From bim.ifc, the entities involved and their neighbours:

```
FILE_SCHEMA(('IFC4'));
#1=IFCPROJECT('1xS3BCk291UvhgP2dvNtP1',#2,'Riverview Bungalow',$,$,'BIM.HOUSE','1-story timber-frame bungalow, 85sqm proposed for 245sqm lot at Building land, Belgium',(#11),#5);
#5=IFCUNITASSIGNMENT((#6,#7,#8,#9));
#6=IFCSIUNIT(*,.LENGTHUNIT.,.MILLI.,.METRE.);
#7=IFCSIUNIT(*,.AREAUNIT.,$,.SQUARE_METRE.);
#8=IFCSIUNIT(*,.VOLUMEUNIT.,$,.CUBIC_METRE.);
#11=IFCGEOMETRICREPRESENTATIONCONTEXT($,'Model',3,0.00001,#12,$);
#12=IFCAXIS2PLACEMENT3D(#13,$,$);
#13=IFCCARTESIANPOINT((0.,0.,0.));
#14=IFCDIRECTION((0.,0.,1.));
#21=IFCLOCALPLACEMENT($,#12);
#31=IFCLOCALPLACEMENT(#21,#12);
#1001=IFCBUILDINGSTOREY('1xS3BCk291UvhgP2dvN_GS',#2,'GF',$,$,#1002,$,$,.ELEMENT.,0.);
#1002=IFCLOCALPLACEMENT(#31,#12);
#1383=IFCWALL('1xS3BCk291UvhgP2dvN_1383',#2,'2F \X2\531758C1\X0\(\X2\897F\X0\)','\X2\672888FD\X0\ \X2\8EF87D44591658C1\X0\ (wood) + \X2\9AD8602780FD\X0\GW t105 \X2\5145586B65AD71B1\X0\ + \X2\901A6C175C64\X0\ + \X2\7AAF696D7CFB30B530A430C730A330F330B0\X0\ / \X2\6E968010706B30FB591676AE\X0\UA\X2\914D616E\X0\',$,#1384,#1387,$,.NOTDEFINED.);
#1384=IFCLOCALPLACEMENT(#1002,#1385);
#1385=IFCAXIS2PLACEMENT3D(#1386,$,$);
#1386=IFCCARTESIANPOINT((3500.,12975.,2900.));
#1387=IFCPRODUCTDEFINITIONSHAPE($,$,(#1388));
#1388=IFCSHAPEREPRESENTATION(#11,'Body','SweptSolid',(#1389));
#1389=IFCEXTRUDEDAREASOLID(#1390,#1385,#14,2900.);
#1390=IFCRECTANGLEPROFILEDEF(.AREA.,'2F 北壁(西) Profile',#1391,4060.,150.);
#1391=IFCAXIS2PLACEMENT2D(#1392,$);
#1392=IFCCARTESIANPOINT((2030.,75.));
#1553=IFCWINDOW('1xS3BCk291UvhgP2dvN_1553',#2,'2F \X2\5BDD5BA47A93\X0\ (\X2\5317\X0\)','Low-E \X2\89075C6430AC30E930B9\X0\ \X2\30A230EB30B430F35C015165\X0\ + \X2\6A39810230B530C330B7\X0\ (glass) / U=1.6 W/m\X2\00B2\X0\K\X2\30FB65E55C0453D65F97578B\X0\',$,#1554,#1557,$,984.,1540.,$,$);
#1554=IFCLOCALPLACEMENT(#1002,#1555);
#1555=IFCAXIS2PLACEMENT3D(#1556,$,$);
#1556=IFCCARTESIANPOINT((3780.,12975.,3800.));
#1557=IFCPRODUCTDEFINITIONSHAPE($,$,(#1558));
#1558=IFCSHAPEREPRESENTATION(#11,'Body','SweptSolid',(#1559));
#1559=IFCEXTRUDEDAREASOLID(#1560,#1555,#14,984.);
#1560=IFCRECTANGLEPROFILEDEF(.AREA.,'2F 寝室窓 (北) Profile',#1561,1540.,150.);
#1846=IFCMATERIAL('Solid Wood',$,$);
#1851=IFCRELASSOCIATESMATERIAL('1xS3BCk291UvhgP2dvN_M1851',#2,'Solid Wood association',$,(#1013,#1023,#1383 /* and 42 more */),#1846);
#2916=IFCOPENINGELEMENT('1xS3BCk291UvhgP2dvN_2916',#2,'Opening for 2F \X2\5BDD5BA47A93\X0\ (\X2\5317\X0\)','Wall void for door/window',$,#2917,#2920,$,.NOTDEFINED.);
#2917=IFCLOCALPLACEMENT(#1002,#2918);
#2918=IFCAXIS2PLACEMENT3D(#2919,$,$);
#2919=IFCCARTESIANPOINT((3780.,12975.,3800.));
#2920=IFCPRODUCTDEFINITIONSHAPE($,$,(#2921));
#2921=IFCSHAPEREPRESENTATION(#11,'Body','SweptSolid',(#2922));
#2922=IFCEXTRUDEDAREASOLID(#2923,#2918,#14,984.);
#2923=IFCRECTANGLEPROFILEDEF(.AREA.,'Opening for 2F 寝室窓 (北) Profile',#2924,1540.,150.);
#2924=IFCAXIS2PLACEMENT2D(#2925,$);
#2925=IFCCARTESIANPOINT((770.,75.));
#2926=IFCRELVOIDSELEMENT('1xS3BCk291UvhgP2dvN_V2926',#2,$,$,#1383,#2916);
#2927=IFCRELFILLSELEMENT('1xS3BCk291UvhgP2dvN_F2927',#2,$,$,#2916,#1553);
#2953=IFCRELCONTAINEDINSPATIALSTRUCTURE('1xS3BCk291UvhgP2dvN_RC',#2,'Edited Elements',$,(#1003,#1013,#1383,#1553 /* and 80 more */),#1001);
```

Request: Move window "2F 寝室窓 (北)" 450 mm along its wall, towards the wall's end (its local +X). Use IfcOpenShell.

```python
import ifcopenshell
import ifcopenshell.api.geometry
import ifcopenshell.util.placement
import ifcopenshell.util.unit

model = ifcopenshell.open("bim.ifc")
unit_scale = ifcopenshell.util.unit.calculate_unit_scale(model)

window = model.by_guid("1xS3BCk291UvhgP2dvN_1553")
opening = window.FillsVoids[0].RelatingOpeningElement
wall = opening.VoidsElements[0].RelatingBuildingElement

wall_matrix = ifcopenshell.util.placement.get_local_placement(wall.ObjectPlacement)
shift = wall_matrix[:3, 0] * 0.45 / unit_scale
before = ifcopenshell.util.placement.get_local_placement(window.ObjectPlacement)[:3, 3].copy()

# The window is not placed relative to its opening, so move both.
for product in (opening, window):
    matrix = ifcopenshell.util.placement.get_local_placement(product.ObjectPlacement)
    matrix[:3, 3] += shift
    ifcopenshell.api.geometry.edit_object_placement(model, product=product, matrix=matrix, is_si=False)

after = ifcopenshell.util.placement.get_local_placement(window.ObjectPlacement)[:3, 3]
print("window moved by", (after - before).round(3) + 0.0)

model.write("bim_updated.ifc")
```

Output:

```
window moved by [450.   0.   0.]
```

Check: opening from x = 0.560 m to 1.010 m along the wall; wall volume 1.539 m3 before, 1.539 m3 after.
